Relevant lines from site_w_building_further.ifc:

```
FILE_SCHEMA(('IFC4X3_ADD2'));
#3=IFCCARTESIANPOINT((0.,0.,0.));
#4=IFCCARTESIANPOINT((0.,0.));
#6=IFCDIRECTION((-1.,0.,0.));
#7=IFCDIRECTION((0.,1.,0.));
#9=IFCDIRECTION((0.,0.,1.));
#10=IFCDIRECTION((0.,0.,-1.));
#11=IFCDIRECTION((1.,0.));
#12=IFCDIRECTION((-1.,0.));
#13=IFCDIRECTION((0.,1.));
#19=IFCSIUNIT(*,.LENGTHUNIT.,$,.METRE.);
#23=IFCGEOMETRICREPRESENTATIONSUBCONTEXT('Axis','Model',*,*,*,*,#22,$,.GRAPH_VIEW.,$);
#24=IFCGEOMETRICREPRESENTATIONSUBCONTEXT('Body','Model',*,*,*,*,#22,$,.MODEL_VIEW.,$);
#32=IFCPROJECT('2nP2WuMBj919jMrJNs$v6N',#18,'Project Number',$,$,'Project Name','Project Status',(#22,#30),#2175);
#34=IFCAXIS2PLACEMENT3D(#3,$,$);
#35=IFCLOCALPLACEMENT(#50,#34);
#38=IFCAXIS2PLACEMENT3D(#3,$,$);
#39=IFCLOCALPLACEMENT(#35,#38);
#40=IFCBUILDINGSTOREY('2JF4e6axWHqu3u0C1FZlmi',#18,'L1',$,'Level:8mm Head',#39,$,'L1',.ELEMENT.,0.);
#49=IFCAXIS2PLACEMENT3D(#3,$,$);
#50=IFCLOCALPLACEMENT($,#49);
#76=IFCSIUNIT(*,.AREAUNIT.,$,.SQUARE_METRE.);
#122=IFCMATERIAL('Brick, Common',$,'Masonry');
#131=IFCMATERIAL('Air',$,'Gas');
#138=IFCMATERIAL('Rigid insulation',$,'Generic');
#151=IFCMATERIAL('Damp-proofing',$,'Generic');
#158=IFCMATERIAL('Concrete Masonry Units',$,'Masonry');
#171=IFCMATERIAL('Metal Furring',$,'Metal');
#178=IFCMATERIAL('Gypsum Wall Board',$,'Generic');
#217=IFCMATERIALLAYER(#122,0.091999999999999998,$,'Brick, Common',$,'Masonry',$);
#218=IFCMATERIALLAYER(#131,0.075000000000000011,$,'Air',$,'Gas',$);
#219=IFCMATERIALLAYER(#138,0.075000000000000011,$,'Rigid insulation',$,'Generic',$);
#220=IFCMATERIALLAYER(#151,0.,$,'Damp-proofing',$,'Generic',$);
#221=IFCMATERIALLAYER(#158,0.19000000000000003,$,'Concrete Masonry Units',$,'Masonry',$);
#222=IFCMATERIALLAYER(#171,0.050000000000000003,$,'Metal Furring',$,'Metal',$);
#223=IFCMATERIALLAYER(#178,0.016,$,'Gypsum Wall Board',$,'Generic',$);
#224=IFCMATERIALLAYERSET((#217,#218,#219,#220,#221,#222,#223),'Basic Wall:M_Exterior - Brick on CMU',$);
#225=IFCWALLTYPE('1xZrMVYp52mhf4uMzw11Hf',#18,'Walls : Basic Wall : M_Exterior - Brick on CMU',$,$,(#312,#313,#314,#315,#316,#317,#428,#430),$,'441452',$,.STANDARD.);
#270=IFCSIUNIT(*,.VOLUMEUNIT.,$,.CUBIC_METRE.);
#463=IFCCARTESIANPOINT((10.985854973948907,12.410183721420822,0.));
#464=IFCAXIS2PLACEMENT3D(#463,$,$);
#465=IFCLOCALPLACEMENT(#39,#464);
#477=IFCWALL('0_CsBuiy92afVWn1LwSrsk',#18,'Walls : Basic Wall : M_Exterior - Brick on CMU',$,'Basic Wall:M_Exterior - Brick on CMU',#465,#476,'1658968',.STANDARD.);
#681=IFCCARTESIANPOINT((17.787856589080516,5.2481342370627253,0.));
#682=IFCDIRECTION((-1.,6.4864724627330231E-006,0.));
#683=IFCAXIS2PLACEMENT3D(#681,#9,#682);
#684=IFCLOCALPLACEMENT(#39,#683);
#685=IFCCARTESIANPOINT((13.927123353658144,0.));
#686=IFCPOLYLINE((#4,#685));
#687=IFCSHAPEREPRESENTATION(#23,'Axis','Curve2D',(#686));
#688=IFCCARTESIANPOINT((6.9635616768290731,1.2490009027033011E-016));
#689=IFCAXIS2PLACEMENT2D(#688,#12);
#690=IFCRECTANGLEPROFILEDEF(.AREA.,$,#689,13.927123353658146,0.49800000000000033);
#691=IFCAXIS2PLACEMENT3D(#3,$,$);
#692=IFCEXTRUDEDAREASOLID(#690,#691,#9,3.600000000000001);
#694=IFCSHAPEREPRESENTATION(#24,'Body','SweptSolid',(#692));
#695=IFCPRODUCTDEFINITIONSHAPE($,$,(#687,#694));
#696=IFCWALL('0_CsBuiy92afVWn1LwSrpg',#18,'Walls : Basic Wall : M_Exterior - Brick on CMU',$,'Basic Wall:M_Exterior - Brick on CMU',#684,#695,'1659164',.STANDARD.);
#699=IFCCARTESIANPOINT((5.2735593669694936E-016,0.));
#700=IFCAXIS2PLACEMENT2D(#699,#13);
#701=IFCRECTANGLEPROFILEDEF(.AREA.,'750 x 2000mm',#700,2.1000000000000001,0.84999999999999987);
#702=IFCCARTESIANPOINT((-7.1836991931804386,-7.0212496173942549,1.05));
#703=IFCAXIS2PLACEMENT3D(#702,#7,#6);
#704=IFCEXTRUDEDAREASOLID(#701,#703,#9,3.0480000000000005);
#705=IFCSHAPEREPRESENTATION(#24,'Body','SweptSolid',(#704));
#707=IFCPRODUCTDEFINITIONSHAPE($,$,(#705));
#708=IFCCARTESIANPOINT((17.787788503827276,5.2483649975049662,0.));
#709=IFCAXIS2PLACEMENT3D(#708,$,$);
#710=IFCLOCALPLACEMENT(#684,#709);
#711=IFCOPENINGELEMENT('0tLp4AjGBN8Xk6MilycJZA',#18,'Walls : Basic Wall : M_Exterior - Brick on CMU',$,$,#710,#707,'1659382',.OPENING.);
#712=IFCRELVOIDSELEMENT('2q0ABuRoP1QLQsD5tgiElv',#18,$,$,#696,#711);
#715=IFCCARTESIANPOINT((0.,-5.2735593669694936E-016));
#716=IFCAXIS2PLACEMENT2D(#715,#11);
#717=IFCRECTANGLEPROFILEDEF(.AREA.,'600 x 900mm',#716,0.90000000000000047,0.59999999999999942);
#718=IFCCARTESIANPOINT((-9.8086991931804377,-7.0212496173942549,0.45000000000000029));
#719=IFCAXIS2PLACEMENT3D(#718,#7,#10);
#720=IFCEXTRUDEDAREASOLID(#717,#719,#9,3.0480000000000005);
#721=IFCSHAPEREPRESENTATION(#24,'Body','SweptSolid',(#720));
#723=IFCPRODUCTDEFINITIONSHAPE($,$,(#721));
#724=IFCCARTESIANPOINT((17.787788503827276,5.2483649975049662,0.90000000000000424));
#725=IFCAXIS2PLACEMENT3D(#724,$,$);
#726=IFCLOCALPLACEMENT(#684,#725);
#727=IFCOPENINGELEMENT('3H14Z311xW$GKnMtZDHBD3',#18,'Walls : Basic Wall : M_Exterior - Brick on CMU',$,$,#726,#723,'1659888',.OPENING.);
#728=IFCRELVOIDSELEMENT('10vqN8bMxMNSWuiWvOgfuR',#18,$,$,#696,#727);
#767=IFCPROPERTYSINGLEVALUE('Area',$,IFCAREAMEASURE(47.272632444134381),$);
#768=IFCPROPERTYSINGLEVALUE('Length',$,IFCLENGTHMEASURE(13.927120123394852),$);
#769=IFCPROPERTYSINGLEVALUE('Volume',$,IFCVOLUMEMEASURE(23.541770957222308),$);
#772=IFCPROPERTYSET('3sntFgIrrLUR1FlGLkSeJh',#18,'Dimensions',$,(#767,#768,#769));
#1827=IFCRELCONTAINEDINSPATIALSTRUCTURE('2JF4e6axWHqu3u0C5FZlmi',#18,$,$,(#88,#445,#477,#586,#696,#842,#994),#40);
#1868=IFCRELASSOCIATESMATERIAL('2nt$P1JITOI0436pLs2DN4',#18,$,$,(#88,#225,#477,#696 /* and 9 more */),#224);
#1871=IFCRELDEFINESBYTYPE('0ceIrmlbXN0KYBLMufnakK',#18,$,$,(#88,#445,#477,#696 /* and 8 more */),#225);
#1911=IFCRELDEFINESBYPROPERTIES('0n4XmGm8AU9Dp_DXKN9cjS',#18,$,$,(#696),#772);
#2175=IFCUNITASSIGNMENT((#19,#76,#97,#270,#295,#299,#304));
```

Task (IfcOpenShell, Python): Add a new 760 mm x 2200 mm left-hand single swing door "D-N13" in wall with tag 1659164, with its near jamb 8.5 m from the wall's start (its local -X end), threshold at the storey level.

```python
import numpy as np
import ifcopenshell
import ifcopenshell.api.feature
import ifcopenshell.api.geometry
import ifcopenshell.api.pset
import ifcopenshell.api.root
import ifcopenshell.api.spatial
import ifcopenshell.geom
import ifcopenshell.util.element
import ifcopenshell.util.placement
import ifcopenshell.util.representation
import ifcopenshell.util.shape
import ifcopenshell.util.unit

model = ifcopenshell.open("site_w_building_further.ifc")
unit_scale = ifcopenshell.util.unit.calculate_unit_scale(model)
area_scale = ifcopenshell.util.unit.calculate_unit_scale(model, "AREAUNIT")
volume_scale = ifcopenshell.util.unit.calculate_unit_scale(model, "VOLUMEUNIT")
settings = ifcopenshell.geom.settings()


def volume(element):
    """Net volume in cubic metres, openings subtracted."""
    shape = ifcopenshell.geom.create_shape(settings, element)
    return ifcopenshell.util.shape.get_volume(shape.geometry)


wall = model.by_id(696)
storey = ifcopenshell.util.element.get_container(wall, ifc_class="IfcBuildingStorey")
context = ifcopenshell.util.representation.get_context(model, "Model", "Body", "MODEL_VIEW")
before = volume(wall)

width, height, from_end, sill = 0.76, 2.2, 8.5, 0.0  # metres

# The wall runs along its own X axis, and the end named is its -X end.
wall_shape = ifcopenshell.geom.create_shape(settings, wall)
x, y, z = ifcopenshell.util.shape.get_vertices(wall_shape.geometry).T
start = x.min() + from_end
face, thickness = float(y.min()), float(y.max() - y.min())
wall_matrix = ifcopenshell.util.placement.get_local_placement(wall.ObjectPlacement)
level = ifcopenshell.util.placement.get_local_placement(storey.ObjectPlacement)[2, 3]


def in_wall(x, y):
    """Placement at x, y metres in the wall's axes, at sill height."""
    matrix = wall_matrix.copy()
    matrix[:, 3] = wall_matrix @ np.array([x / unit_scale, y / unit_scale, 0.0, 1.0])
    matrix[2, 3] = level + sill / unit_scale
    return matrix


# Opening: a box that overshoots both wall faces by 50 mm.
opening = ifcopenshell.api.root.create_entity(model, ifc_class="IfcOpeningElement", predefined_type="OPENING")
box = ifcopenshell.api.geometry.add_wall_representation(
    model, context=context, length=width, height=height, thickness=thickness + 0.1
)
ifcopenshell.api.geometry.assign_representation(model, product=opening, representation=box)
ifcopenshell.api.geometry.edit_object_placement(model, product=opening, matrix=in_wall(start, face - 0.05), is_si=False)
ifcopenshell.api.feature.add_feature(model, feature=opening, element=wall)

door = ifcopenshell.api.root.create_entity(model, ifc_class="IfcDoor", name="D-N13", predefined_type="DOOR")
door.OverallWidth, door.OverallHeight = width / unit_scale, height / unit_scale
door.OperationType = "SINGLE_SWING_LEFT"
body = ifcopenshell.api.geometry.add_door_representation(
    model,
    context=context,
    overall_width=door.OverallWidth,
    overall_height=door.OverallHeight,
    operation_type="SINGLE_SWING_LEFT",
    lining_properties={"LiningDepth": thickness / unit_scale, "ThresholdDepth": thickness / unit_scale},
)
ifcopenshell.api.geometry.assign_representation(model, product=door, representation=body)
ifcopenshell.api.spatial.assign_container(model, products=[door], relating_structure=storey)
ifcopenshell.api.feature.add_filling(model, opening=opening, element=door)

# The lining spans the wall, so the door starts at the wall face.
ifcopenshell.api.geometry.edit_object_placement(model, product=door, matrix=in_wall(start, face), is_si=False)

after = volume(wall)

# Update the wall's stored quantities.
pset = model.by_id(ifcopenshell.util.element.get_pset(wall, "Dimensions", should_inherit=False)["id"])
ifcopenshell.api.pset.edit_pset(model, pset=pset, properties={
    "Area": model.create_entity("IfcAreaMeasure", after / thickness / area_scale),
    "Volume": model.create_entity("IfcVolumeMeasure", after / volume_scale),
})

print(f"wall volume {before:.3f} -> {after:.3f} m3")

model.write("site_w_building_further_edited.ifc")
```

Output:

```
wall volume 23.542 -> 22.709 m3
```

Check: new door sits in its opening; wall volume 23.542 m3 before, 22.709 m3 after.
